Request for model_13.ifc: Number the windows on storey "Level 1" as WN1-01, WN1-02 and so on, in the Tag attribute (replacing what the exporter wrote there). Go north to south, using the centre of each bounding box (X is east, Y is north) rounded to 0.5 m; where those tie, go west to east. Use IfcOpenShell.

First a look at what the model holds.

```python
import ifcopenshell
import ifcopenshell.util.element
import ifcopenshell.util.placement

model = ifcopenshell.open("model_13.ifc")
print(model.schema)
storey = next(s for s in model.by_type("IfcBuildingStorey") if s.Name == "Level 1")
windows = [e for e in ifcopenshell.util.element.get_decomposition(storey) if e.is_a("IfcWindow")]
for e in sorted(windows, key=lambda e: e.id()):
    origin = ifcopenshell.util.placement.get_local_placement(e.ObjectPlacement)[:3, 3]
    print(e.id(), e.Tag, e.Name, origin.round(2) + 0.0, sep=" | ")
```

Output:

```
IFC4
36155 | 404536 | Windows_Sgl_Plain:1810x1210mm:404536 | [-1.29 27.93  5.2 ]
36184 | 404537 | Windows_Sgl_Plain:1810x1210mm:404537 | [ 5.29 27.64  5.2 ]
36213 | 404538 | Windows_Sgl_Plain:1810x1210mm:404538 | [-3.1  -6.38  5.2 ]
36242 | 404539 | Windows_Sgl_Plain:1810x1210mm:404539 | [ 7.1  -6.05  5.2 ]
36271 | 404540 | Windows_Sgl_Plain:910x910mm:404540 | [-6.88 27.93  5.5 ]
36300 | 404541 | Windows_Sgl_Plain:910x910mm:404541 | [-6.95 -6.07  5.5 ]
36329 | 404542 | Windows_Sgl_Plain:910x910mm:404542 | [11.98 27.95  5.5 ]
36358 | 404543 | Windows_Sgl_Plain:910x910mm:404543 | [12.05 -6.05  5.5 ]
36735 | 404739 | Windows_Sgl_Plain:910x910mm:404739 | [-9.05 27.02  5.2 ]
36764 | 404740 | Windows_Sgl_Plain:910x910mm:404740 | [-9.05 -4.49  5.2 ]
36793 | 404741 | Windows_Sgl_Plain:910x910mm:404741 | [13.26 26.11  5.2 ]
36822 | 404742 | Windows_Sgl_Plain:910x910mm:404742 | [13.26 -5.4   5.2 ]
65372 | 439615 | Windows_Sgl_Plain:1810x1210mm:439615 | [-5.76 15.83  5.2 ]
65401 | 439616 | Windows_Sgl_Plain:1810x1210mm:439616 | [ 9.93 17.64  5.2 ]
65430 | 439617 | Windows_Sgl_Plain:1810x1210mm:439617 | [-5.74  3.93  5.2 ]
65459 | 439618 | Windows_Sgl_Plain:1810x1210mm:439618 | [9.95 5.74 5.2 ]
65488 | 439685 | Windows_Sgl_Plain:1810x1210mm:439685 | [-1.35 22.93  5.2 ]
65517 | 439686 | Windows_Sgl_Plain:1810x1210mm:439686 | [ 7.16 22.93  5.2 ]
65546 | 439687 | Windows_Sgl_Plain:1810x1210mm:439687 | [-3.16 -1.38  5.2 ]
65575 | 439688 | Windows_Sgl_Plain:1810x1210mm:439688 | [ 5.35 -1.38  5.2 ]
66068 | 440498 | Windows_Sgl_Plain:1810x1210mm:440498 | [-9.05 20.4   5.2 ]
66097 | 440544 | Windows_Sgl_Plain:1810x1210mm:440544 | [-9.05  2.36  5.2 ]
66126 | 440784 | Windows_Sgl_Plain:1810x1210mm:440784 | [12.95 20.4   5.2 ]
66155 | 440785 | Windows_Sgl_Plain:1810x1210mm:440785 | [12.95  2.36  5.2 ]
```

```python
import ifcopenshell
import ifcopenshell.geom
import ifcopenshell.util.element
import ifcopenshell.util.shape

model = ifcopenshell.open("model_13.ifc")
settings = ifcopenshell.geom.settings()
settings.set("use-world-coords", True)


def centre(element):
    shape = ifcopenshell.geom.create_shape(settings, element)
    return ifcopenshell.util.shape.get_bbox_centroid(shape.geometry)


storey = next(s for s in model.by_type("IfcBuildingStorey") if s.Name == "Level 1")
windows = [e for e in ifcopenshell.util.element.get_decomposition(storey) if e.is_a("IfcWindow")]

# Insertion points can sit at a corner or the storey origin, so sort by the geometry (in metres).
centres = {e: centre(e) for e in windows}
windows.sort(key=lambda e: (-round(centres[e][1] / 0.5), centres[e][0]))

for i, e in enumerate(windows, start=1):
    number = f"WN1-{i:02d}"
    e.Tag = number
    print(e.id(), number)

model.write("model_13_updated.ifc")
```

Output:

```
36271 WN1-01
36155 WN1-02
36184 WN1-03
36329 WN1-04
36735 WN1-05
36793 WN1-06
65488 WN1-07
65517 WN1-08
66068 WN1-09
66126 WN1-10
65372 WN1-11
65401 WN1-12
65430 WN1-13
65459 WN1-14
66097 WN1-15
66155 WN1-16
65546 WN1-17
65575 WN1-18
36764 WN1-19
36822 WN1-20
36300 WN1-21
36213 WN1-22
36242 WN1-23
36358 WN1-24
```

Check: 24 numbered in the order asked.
